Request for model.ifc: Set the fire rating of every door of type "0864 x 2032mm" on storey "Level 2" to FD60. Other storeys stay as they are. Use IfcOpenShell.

First a look at what the model holds.

```python
import ifcopenshell
import ifcopenshell.util.element

model = ifcopenshell.open("model.ifc")
print(model.schema)
storey = next(s for s in model.by_type("IfcBuildingStorey") if s.Name == "Level 2")
doors = [e for e in ifcopenshell.util.element.get_decomposition(storey) if e.is_a("IfcDoor")]
seen = {}
for e in doors:
    element_type = ifcopenshell.util.element.get_type(e)
    key = (element_type.Name if element_type != e and element_type else None, ifcopenshell.util.element.get_pset(e, "Pset_DoorCommon", "FireRating"))
    seen[key] = seen.get(key, 0) + 1
for (name, value), count in sorted(seen.items(), key=str):
    print(count, "x", name, "|", value)
```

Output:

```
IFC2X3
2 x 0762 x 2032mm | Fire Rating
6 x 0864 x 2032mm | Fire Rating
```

```python
import ifcopenshell
import ifcopenshell.api.pset
import ifcopenshell.util.element

model = ifcopenshell.open("model.ifc")

storey = next(s for s in model.by_type("IfcBuildingStorey") if s.Name == "Level 2")
doors = [e for e in ifcopenshell.util.element.get_decomposition(storey) if e.is_a("IfcDoor")]

count = 0
for e in doors:
    element_type = ifcopenshell.util.element.get_type(e)
    if element_type in (None, e) or element_type.Name != "0864 x 2032mm":
        continue
    # add_pset returns the element's existing set when there is one.
    pset = ifcopenshell.api.pset.add_pset(model, product=e, name="Pset_DoorCommon")
    ifcopenshell.api.pset.edit_pset(model, pset=pset, properties={"FireRating": "FD60"})
    count += 1

print(count, "doors updated")

model.write("model-out.ifc")
```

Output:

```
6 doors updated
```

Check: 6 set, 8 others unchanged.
